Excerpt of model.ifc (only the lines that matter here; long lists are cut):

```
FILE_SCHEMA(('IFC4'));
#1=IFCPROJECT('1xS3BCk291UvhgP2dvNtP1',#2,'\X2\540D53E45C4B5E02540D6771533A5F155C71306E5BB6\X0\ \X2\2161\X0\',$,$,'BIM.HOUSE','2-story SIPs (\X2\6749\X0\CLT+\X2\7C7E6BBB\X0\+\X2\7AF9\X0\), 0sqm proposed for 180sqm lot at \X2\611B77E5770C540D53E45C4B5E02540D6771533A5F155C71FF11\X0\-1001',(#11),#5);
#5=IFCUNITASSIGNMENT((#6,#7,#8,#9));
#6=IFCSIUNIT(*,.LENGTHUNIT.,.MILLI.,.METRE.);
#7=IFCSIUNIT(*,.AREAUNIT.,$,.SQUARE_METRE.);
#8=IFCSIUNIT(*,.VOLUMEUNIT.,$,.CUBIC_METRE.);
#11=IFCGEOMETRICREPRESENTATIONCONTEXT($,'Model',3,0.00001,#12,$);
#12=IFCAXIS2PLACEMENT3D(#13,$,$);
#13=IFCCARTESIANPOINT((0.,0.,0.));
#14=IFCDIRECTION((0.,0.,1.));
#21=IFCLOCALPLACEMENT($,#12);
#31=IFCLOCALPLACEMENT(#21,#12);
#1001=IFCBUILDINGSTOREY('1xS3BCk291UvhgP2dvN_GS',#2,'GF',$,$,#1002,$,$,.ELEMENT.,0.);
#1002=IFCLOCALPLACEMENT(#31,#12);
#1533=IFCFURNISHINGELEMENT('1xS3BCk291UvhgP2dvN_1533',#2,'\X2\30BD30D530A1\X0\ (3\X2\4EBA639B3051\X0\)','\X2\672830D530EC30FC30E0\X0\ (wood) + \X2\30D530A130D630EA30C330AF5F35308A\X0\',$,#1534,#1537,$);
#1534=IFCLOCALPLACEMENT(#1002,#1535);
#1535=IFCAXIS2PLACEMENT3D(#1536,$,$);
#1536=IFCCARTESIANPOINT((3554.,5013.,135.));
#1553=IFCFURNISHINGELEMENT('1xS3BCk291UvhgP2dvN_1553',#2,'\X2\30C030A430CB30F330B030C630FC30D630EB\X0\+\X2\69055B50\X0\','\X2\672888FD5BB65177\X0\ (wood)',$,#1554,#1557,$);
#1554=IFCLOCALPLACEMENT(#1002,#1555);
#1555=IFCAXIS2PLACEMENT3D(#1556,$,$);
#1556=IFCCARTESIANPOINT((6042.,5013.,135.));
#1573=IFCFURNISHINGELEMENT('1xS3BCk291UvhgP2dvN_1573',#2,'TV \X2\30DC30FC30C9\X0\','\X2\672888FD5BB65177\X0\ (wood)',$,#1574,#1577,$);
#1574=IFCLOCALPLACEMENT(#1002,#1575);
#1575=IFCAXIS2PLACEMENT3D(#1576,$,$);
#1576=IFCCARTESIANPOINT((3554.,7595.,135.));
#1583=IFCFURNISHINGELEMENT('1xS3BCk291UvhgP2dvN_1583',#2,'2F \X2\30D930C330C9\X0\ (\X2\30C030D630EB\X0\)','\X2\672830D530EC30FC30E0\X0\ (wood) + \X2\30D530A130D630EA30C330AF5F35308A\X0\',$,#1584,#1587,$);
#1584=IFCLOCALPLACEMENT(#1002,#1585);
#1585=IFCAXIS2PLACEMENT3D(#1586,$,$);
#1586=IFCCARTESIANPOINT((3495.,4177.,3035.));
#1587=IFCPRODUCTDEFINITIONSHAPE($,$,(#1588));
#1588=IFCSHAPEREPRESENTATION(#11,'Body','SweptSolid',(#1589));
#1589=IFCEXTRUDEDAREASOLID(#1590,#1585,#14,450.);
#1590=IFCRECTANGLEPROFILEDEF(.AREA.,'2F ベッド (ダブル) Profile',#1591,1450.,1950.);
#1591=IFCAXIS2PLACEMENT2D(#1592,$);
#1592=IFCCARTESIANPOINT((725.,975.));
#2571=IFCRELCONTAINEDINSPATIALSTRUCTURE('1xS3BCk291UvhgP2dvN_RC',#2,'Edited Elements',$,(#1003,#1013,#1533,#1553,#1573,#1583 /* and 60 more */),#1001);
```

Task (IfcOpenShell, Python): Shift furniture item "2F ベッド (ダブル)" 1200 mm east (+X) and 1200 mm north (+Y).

```python
import ifcopenshell
import ifcopenshell.api.geometry
import ifcopenshell.util.placement
import ifcopenshell.util.unit

model = ifcopenshell.open("model.ifc")
unit_scale = ifcopenshell.util.unit.calculate_unit_scale(model)

item = model.by_guid("1xS3BCk291UvhgP2dvN_1583")
matrix = ifcopenshell.util.placement.get_local_placement(item.ObjectPlacement)
matrix[0, 3] += 1.2 / unit_scale
matrix[1, 3] += 1.2 / unit_scale
ifcopenshell.api.geometry.edit_object_placement(model, product=item, matrix=matrix, is_si=False)

print(ifcopenshell.util.placement.get_local_placement(item.ObjectPlacement).round(3) + 0.0)

model.write("model_rev.ifc")
```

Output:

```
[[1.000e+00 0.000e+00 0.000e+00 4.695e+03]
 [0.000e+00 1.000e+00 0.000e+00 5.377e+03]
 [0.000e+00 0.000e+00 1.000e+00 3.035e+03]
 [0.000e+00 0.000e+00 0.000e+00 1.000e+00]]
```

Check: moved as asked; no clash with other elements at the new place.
